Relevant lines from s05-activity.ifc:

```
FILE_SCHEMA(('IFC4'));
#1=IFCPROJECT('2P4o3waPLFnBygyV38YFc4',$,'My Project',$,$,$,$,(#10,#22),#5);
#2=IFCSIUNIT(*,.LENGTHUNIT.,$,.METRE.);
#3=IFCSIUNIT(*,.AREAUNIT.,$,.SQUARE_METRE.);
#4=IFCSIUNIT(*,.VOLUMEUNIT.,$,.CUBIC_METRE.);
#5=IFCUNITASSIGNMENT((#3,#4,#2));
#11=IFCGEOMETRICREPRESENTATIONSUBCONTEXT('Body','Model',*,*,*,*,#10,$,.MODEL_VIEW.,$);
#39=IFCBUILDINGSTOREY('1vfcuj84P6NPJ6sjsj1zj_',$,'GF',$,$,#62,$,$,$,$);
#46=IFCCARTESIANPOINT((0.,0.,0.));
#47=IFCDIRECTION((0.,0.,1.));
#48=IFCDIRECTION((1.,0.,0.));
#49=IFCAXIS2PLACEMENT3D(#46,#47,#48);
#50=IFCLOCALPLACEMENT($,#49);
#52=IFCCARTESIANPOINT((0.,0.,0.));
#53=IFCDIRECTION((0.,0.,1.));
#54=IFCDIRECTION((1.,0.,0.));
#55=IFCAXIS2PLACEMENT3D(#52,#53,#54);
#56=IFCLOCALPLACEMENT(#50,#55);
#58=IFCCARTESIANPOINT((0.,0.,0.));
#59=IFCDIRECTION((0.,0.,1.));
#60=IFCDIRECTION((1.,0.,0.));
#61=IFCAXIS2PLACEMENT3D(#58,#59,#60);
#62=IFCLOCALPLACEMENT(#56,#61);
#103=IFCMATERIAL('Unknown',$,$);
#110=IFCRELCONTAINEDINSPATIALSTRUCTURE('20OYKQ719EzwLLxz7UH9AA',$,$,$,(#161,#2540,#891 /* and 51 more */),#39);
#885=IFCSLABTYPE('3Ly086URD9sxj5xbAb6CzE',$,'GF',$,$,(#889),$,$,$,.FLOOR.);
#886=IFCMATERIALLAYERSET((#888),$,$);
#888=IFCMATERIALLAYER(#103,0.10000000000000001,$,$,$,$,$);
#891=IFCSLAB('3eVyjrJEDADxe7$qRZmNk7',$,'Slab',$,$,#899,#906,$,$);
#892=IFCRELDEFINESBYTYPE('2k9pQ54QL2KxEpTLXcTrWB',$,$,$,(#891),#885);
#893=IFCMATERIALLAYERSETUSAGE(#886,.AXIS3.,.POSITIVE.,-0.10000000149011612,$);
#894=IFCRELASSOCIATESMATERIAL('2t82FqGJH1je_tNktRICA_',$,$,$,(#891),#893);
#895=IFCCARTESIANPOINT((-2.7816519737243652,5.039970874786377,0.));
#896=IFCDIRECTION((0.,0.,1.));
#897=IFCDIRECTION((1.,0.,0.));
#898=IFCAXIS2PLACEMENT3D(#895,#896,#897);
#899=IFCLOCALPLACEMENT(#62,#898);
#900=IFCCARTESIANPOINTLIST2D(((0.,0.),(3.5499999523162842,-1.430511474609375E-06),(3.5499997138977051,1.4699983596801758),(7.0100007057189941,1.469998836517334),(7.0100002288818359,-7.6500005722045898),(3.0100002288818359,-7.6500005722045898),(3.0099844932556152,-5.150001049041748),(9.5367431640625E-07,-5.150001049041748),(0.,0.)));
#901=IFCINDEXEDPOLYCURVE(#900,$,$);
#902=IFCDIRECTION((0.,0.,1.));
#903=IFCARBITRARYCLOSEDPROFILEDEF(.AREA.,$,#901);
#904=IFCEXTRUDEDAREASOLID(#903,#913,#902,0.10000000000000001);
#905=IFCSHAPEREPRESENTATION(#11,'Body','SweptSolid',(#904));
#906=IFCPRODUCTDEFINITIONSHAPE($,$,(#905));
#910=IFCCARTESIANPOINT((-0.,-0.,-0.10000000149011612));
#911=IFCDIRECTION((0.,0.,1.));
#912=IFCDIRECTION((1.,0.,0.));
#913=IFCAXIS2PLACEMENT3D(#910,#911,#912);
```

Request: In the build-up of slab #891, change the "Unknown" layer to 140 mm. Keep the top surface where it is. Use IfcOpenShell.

```python
import ifcopenshell
import ifcopenshell.util.element
import ifcopenshell.util.representation

model = ifcopenshell.open("s05-activity.ifc")

layer_set = model.by_id(886)
layer = next(l for l in layer_set.MaterialLayers if l.Material and l.Material.Name == "Unknown")
change = 0.14 - layer.LayerThickness
layer.LayerThickness += change

# Geometry does not follow the layer set by itself.
slabs = [e for e in ifcopenshell.util.element.get_elements_by_material(model, layer_set) if e.is_a("IfcSlab")]
for slab in sorted(slabs, key=lambda e: e.id()):
    body = ifcopenshell.util.representation.get_representation(slab, "Model", "Body")
    solid = body.Items[0]
    old_depth = solid.Depth
    solid.Depth += change
    # Extruded upwards: lower the start of the extrusion so the top stays.
    x, y, z = solid.Position.Location.Coordinates
    solid.Position.Location = model.createIfcCartesianPoint((x, y, z - change))
    print(slab.id(), f"{old_depth:g} -> {solid.Depth:g}")

# The layers are counted up from the underside, which has moved.
for usage in {ifcopenshell.util.element.get_material(slab) for slab in slabs}:
    usage.OffsetFromReferenceLine -= change

model.write("s05-activity_edited.ifc")
```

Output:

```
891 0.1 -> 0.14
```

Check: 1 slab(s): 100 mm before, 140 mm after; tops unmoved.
